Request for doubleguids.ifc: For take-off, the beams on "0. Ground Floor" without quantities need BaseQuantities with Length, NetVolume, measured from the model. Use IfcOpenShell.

First a look at what the model holds.

```python
import ifcopenshell
import ifcopenshell.util.element
import ifcopenshell.util.unit

model = ifcopenshell.open("doubleguids.ifc")
print(model.schema)
for unit_type in ("LENGTHUNIT", "AREAUNIT", "VOLUMEUNIT"):
    print(unit_type, ifcopenshell.util.unit.calculate_unit_scale(model, unit_type))
storey = next(s for s in model.by_type("IfcBuildingStorey") if s.Name == "0. Ground Floor")
beams = [e for e in ifcopenshell.util.element.get_decomposition(storey) if e.is_a("IfcBeam")]
for e in sorted(beams, key=lambda e: e.id()):
    print(e.id(), e.is_a(), e.Name, list(ifcopenshell.util.element.get_psets(e, qtos_only=True)), sep=" | ")
```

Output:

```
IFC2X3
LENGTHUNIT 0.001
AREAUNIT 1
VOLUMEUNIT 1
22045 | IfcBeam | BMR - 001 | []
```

```python
import ifcopenshell
import ifcopenshell.api.pset
import ifcopenshell.geom
import ifcopenshell.util.element
import ifcopenshell.util.shape
import ifcopenshell.util.unit

model = ifcopenshell.open("doubleguids.ifc")
unit_scale = ifcopenshell.util.unit.calculate_unit_scale(model)
volume_scale = ifcopenshell.util.unit.calculate_unit_scale(model, "VOLUMEUNIT")
settings = ifcopenshell.geom.settings()

storey = next(s for s in model.by_type("IfcBuildingStorey") if s.Name == "0. Ground Floor")
beams = [e for e in ifcopenshell.util.element.get_decomposition(storey) if e.is_a("IfcBeam")]

for e in sorted(beams, key=lambda e: e.id()):
    if ifcopenshell.util.element.get_psets(e, qtos_only=True, should_inherit=False):
        continue
    # Geometry comes back in metres, in the element's own axes.
    shape = ifcopenshell.geom.create_shape(settings, e)
    values = {
        "Length": ifcopenshell.util.shape.get_max_xyz(shape.geometry) / unit_scale,
        "NetVolume": ifcopenshell.util.shape.get_volume(shape.geometry) / volume_scale,
    }
    qto = ifcopenshell.api.pset.add_qto(model, product=e, name="BaseQuantities")
    ifcopenshell.api.pset.edit_qto(model, qto=qto, properties=values)
    print(e.id(), {k: round(v, 3) for k, v in values.items()})

model.write("doubleguids_rev.ifc")
```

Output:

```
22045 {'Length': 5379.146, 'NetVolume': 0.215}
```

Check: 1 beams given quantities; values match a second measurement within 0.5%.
